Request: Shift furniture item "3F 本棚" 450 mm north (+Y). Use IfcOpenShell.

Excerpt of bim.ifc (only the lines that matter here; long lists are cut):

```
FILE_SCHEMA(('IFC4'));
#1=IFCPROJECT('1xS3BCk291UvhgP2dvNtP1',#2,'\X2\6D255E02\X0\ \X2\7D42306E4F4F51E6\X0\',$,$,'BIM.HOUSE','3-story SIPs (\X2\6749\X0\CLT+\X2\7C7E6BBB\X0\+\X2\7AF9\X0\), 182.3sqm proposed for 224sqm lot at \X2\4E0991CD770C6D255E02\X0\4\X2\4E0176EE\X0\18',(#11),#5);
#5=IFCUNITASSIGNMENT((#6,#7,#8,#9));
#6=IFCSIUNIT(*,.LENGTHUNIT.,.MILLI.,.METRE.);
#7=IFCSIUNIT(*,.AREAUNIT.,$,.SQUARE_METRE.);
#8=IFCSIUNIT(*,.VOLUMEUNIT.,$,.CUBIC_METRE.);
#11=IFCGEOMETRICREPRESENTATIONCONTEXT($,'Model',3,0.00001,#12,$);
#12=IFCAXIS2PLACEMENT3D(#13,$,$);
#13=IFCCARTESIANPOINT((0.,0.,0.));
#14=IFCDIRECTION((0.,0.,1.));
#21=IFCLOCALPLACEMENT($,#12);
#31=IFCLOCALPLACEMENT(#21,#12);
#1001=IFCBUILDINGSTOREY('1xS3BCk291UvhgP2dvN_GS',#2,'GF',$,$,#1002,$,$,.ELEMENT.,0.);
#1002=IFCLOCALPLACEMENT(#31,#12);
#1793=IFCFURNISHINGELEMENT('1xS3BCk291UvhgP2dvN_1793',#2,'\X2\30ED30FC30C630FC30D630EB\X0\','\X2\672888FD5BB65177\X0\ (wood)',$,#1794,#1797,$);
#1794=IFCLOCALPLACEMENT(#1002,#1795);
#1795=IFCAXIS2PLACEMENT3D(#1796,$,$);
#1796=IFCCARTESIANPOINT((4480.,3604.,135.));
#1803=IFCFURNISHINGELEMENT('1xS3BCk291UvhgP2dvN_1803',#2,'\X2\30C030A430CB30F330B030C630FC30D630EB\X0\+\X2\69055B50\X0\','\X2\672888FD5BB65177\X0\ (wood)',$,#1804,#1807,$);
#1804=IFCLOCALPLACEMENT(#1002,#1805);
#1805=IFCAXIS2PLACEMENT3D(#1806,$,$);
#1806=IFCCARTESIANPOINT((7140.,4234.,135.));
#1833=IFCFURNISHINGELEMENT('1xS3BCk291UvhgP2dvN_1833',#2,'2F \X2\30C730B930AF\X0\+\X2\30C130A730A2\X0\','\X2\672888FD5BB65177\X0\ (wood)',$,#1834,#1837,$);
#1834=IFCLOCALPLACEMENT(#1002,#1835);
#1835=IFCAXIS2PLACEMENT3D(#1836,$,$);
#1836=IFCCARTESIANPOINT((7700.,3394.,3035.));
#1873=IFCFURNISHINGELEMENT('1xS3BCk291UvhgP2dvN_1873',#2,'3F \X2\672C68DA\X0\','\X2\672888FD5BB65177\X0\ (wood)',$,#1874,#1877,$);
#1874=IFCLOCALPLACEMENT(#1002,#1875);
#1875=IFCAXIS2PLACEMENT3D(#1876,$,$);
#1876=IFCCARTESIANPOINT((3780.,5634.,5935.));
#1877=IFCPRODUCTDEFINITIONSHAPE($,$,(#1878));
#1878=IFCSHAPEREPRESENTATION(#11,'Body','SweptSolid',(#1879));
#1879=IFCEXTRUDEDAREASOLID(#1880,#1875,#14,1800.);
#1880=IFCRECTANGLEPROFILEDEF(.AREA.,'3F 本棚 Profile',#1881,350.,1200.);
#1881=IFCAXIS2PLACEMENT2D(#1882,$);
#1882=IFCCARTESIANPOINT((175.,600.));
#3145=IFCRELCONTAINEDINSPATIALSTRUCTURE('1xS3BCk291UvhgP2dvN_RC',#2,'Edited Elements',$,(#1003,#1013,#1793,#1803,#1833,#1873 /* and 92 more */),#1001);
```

```python
import ifcopenshell
import ifcopenshell.api.geometry
import ifcopenshell.util.placement
import ifcopenshell.util.unit

model = ifcopenshell.open("bim.ifc")
unit_scale = ifcopenshell.util.unit.calculate_unit_scale(model)

item = model.by_guid("1xS3BCk291UvhgP2dvN_1873")
matrix = ifcopenshell.util.placement.get_local_placement(item.ObjectPlacement)
matrix[1, 3] += 0.45 / unit_scale
ifcopenshell.api.geometry.edit_object_placement(model, product=item, matrix=matrix, is_si=False)

print(ifcopenshell.util.placement.get_local_placement(item.ObjectPlacement).round(3) + 0.0)

model.write("bim_updated.ifc")
```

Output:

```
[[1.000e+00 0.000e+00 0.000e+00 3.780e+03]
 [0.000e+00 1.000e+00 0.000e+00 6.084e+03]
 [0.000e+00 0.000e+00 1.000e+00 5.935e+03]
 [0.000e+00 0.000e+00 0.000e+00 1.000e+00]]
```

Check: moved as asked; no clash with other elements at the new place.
